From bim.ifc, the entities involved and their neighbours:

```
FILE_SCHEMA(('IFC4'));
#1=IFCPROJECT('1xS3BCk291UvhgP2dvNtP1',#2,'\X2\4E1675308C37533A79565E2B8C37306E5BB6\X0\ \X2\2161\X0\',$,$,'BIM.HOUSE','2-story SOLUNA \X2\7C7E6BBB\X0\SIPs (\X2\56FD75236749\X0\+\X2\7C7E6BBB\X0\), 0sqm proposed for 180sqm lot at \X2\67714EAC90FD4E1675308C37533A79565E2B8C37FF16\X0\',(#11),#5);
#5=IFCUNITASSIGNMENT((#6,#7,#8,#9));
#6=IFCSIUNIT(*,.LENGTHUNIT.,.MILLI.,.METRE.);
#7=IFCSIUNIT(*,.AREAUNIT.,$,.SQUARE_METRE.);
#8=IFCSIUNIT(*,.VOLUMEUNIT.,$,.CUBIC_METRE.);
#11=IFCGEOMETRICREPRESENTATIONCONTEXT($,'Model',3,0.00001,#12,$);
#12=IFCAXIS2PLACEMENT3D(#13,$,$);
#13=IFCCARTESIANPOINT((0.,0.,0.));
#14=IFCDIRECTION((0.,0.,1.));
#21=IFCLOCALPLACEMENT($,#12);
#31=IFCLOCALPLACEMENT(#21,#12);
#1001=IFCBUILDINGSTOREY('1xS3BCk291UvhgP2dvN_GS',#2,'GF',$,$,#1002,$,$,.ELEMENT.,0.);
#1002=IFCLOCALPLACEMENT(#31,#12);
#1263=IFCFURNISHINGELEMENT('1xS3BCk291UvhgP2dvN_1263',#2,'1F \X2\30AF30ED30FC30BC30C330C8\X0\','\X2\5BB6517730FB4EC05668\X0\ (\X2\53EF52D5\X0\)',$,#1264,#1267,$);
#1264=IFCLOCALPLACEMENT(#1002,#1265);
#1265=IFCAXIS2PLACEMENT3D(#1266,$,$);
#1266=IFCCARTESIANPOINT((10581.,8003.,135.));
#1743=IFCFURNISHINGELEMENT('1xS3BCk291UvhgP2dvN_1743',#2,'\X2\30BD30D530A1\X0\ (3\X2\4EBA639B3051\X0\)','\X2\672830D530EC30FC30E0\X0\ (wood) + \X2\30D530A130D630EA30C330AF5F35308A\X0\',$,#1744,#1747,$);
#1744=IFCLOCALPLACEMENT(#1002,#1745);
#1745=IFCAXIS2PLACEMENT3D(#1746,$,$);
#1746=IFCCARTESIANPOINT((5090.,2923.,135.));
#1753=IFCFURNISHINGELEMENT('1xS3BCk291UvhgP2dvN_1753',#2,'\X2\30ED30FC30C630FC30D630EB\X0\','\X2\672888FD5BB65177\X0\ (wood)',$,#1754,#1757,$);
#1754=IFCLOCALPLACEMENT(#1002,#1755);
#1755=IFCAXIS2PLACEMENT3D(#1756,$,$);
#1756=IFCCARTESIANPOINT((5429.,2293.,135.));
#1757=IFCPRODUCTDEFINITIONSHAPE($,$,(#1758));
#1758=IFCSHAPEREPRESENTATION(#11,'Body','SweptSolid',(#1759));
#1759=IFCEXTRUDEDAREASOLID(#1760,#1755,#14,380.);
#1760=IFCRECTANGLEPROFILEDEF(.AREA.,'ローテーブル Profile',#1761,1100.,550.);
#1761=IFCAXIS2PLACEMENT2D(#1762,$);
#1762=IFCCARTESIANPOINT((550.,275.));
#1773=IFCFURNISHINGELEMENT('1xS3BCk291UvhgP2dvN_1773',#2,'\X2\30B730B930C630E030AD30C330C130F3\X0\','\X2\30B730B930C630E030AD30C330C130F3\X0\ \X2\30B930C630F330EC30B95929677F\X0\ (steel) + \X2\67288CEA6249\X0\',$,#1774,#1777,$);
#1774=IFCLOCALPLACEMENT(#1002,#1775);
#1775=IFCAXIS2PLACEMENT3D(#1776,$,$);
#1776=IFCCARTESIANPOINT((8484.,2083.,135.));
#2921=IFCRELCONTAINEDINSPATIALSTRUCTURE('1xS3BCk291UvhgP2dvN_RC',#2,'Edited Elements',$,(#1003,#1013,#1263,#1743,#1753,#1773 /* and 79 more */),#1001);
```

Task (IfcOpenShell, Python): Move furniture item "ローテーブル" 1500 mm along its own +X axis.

```python
import ifcopenshell
import ifcopenshell.api.geometry
import ifcopenshell.util.placement
import ifcopenshell.util.unit

model = ifcopenshell.open("bim.ifc")
unit_scale = ifcopenshell.util.unit.calculate_unit_scale(model)

item = model.by_id(1753)
matrix = ifcopenshell.util.placement.get_local_placement(item.ObjectPlacement)
matrix[:3, 3] += matrix[:3, 0] * 1.5 / unit_scale
ifcopenshell.api.geometry.edit_object_placement(model, product=item, matrix=matrix, is_si=False)

print(ifcopenshell.util.placement.get_local_placement(item.ObjectPlacement).round(3) + 0.0)

model.write("bim_edited.ifc")
```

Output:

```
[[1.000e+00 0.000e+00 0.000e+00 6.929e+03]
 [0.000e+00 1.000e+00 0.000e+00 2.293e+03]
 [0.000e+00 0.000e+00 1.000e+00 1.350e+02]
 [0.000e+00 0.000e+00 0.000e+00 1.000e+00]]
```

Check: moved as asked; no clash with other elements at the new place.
